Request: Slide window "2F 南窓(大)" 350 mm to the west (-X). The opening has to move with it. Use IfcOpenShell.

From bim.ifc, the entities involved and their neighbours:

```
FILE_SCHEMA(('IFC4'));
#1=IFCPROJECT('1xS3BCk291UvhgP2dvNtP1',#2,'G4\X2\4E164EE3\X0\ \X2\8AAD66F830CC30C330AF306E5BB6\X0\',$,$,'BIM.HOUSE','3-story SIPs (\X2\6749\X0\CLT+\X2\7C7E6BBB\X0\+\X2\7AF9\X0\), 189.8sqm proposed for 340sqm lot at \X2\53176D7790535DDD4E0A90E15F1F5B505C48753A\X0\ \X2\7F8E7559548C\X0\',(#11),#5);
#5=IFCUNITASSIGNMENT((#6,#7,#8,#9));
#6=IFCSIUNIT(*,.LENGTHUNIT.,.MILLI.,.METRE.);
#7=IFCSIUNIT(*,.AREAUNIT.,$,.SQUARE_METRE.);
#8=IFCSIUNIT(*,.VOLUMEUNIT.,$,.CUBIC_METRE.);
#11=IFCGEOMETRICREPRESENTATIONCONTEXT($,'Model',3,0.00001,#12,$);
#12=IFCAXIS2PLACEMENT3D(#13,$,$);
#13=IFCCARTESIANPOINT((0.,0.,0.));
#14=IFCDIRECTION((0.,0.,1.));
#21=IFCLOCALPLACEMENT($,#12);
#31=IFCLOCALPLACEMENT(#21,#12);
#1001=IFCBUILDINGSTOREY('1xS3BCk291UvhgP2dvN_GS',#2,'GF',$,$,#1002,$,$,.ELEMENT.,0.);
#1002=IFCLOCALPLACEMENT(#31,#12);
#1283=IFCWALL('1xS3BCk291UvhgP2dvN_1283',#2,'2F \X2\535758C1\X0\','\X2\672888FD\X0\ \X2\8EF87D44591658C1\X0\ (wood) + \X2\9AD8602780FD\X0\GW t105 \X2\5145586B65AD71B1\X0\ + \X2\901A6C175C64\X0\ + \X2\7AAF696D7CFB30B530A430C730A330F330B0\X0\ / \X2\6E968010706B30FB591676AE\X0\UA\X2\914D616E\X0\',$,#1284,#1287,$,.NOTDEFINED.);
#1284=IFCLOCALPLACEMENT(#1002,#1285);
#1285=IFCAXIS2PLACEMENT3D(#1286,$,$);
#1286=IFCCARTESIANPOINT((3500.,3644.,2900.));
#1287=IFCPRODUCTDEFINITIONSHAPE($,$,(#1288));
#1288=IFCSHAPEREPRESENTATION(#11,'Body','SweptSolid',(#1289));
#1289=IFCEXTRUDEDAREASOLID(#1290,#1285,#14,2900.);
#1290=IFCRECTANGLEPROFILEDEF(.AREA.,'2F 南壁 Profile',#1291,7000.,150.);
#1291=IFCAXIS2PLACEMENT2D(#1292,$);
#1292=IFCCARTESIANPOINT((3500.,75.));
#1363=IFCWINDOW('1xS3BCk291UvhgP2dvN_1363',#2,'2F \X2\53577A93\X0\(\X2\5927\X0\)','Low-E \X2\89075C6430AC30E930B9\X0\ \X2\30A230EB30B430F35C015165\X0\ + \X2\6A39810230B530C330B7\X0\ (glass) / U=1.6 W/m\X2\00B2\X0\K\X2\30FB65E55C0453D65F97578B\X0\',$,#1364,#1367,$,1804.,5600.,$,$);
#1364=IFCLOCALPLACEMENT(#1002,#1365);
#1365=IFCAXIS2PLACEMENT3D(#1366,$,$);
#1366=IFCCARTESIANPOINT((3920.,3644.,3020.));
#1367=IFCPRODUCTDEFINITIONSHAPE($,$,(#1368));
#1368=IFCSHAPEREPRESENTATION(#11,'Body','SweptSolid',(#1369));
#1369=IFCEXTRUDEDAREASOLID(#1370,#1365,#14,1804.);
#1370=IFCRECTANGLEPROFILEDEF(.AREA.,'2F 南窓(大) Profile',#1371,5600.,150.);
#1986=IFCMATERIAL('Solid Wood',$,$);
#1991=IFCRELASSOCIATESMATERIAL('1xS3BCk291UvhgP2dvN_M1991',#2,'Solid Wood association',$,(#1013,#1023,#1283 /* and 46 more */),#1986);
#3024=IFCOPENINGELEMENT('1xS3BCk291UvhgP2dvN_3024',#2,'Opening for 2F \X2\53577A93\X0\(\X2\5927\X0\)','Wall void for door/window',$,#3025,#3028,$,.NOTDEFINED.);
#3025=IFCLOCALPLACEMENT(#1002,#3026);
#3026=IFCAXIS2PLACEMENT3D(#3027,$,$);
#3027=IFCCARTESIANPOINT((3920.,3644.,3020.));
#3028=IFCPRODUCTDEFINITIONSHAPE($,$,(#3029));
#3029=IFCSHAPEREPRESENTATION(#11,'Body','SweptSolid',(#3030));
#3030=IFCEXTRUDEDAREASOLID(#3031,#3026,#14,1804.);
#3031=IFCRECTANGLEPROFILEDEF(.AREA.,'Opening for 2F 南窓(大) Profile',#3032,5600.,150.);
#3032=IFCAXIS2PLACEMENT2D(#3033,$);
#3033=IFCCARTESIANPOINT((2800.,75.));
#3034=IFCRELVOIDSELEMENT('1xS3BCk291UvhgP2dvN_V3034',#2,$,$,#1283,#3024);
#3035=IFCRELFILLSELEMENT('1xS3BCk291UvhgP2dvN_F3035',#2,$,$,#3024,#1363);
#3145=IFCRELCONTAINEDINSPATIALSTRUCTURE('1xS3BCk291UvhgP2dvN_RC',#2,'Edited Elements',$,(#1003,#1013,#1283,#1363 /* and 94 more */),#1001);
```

```python
import ifcopenshell
import ifcopenshell.api.geometry
import ifcopenshell.util.placement
import ifcopenshell.util.unit

model = ifcopenshell.open("bim.ifc")
unit_scale = ifcopenshell.util.unit.calculate_unit_scale(model)

window = model.by_guid("1xS3BCk291UvhgP2dvN_1363")
opening = window.FillsVoids[0].RelatingOpeningElement
wall = opening.VoidsElements[0].RelatingBuildingElement

wall_matrix = ifcopenshell.util.placement.get_local_placement(wall.ObjectPlacement)
shift = wall_matrix[:3, 0] * -0.35 / unit_scale
before = ifcopenshell.util.placement.get_local_placement(window.ObjectPlacement)[:3, 3].copy()

# The window is not placed relative to its opening, so move both.
for product in (opening, window):
    matrix = ifcopenshell.util.placement.get_local_placement(product.ObjectPlacement)
    matrix[:3, 3] += shift
    ifcopenshell.api.geometry.edit_object_placement(model, product=product, matrix=matrix, is_si=False)

after = ifcopenshell.util.placement.get_local_placement(window.ObjectPlacement)[:3, 3]
print("window moved by", (after - before).round(3) + 0.0)

model.write("bim_v2.ifc")
```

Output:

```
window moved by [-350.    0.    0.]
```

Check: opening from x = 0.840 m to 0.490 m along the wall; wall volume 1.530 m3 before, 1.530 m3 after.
